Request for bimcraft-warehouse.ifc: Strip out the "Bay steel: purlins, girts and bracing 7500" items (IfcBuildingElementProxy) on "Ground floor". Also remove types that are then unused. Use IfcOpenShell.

First a look at what the model holds.

```python
import ifcopenshell
import ifcopenshell.util.element

model = ifcopenshell.open("bimcraft-warehouse.ifc")
print(model.schema)
storey = next(s for s in model.by_type("IfcBuildingStorey") if s.Name == "Ground floor")
proxies = [e for e in ifcopenshell.util.element.get_decomposition(storey) if e.is_a("IfcBuildingElementProxy")]
seen = {}
for e in proxies:
    element_type = ifcopenshell.util.element.get_type(e)
    name = element_type.Name if element_type not in (None, e) else None
    seen[name] = seen.get(name, 0) + 1
for name, count in sorted(seen.items(), key=str):
    print(count, "x", name)
```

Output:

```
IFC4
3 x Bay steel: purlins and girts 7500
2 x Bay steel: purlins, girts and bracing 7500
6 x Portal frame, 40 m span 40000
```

```python
import ifcopenshell
import ifcopenshell.api.root
import ifcopenshell.util.element

model = ifcopenshell.open("bimcraft-warehouse.ifc")

storey = next(s for s in model.by_type("IfcBuildingStorey") if s.Name == "Ground floor")
proxies = [e for e in ifcopenshell.util.element.get_decomposition(storey) if e.is_a("IfcBuildingElementProxy")]
targets = [e for e in proxies if (t := ifcopenshell.util.element.get_type(e)) not in (None, e) and t.Name == "Bay steel: purlins, girts and bracing 7500"]
types = {ifcopenshell.util.element.get_type(e) for e in targets} - {None, *targets}

for e in targets:
    ifcopenshell.api.root.remove_product(model, product=e)
print(len(targets), "removed")

unused = [t for t in types if not ifcopenshell.util.element.get_types(t)]
for t in unused:
    ifcopenshell.api.root.remove_product(model, product=t)
print(len(unused), "unused types removed")

model.write("bimcraft-warehouse_edited.ifc")
```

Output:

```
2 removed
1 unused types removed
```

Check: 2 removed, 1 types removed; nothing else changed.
